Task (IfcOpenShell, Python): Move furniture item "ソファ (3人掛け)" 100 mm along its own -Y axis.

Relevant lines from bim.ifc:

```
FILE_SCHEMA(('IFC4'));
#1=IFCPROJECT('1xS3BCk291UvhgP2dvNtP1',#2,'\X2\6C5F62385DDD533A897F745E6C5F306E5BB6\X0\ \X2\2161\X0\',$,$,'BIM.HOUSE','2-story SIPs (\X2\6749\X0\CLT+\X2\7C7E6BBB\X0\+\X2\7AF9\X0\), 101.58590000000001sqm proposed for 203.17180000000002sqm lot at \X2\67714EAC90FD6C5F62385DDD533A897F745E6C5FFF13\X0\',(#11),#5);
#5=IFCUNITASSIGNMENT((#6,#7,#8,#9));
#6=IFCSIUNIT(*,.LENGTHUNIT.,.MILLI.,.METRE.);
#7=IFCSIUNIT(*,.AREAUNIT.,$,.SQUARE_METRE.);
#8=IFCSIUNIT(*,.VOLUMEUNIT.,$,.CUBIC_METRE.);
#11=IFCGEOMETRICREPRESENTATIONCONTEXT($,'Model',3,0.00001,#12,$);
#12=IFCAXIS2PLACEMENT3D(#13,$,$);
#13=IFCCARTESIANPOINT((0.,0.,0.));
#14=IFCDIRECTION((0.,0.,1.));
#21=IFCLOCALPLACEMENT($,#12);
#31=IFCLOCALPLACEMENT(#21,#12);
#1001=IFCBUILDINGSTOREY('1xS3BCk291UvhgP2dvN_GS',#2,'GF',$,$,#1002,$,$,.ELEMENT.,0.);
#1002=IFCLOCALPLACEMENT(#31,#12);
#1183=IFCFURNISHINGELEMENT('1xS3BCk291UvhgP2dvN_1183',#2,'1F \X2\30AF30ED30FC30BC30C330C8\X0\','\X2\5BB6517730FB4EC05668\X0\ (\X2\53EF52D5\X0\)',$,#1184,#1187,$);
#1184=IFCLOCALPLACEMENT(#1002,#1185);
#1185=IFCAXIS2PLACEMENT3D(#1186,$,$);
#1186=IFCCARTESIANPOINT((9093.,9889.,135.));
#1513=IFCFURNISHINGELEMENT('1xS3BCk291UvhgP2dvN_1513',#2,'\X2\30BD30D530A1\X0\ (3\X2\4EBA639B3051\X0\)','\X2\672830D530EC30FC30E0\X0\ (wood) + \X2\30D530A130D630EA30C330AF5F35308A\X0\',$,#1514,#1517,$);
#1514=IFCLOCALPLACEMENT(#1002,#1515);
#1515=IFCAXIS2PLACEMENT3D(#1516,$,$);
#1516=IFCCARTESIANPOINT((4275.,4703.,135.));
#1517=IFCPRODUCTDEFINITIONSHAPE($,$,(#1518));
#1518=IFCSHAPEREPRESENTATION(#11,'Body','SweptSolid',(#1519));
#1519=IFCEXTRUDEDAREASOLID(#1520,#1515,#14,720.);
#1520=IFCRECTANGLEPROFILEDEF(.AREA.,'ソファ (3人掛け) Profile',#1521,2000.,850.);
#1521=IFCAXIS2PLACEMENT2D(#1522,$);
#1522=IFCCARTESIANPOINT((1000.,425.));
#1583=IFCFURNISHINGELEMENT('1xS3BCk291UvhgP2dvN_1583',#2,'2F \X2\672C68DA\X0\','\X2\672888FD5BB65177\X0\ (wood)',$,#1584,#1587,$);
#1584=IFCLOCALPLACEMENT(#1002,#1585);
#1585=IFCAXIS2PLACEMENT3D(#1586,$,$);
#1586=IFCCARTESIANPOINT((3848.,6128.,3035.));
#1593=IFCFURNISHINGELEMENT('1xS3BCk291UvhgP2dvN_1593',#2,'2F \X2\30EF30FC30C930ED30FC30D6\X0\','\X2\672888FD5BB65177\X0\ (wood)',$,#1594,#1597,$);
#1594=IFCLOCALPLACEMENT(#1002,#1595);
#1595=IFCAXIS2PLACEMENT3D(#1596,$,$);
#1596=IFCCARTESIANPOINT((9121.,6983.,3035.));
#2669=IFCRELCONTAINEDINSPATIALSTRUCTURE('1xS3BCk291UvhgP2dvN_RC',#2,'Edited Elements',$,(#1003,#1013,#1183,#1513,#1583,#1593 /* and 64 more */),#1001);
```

```python
import ifcopenshell
import ifcopenshell.api.geometry
import ifcopenshell.util.placement
import ifcopenshell.util.unit

model = ifcopenshell.open("bim.ifc")
unit_scale = ifcopenshell.util.unit.calculate_unit_scale(model)

item = model.by_id(1513)
matrix = ifcopenshell.util.placement.get_local_placement(item.ObjectPlacement)
matrix[:3, 3] -= matrix[:3, 1] * 0.1 / unit_scale
ifcopenshell.api.geometry.edit_object_placement(model, product=item, matrix=matrix, is_si=False)

print(ifcopenshell.util.placement.get_local_placement(item.ObjectPlacement).round(3) + 0.0)

model.write("bim_updated.ifc")
```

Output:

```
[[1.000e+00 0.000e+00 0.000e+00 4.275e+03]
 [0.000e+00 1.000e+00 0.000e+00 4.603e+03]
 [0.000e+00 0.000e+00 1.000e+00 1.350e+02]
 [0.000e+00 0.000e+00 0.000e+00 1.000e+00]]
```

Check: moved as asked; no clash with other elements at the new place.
